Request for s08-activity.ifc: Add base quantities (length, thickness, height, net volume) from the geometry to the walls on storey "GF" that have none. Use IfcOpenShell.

First a look at what the model holds.

```python
import ifcopenshell
import ifcopenshell.util.element
import ifcopenshell.util.unit

model = ifcopenshell.open("s08-activity.ifc")
print(model.schema)
for unit_type in ("LENGTHUNIT", "AREAUNIT", "VOLUMEUNIT"):
    print(unit_type, ifcopenshell.util.unit.calculate_unit_scale(model, unit_type))
storey = next(s for s in model.by_type("IfcBuildingStorey") if s.Name == "GF")
walls = [e for e in ifcopenshell.util.element.get_decomposition(storey) if e.is_a("IfcWall")]
for e in sorted(walls, key=lambda e: e.id()):
    print(e.id(), e.is_a(), e.Name, list(ifcopenshell.util.element.get_psets(e, qtos_only=True)), sep=" | ")
```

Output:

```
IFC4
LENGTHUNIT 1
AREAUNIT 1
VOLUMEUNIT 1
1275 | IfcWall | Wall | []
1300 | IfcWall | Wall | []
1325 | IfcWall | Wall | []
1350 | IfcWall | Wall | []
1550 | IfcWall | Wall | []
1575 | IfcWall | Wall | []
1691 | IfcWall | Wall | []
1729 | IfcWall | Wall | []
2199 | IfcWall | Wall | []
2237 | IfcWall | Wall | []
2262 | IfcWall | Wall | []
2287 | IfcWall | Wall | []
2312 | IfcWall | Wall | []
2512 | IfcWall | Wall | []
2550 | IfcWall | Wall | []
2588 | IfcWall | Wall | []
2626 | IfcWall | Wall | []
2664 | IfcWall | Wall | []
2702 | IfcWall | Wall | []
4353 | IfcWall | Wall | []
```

```python
import ifcopenshell
import ifcopenshell.api.pset
import ifcopenshell.geom
import ifcopenshell.util.element
import ifcopenshell.util.shape
import ifcopenshell.util.unit

model = ifcopenshell.open("s08-activity.ifc")
unit_scale = ifcopenshell.util.unit.calculate_unit_scale(model)
volume_scale = ifcopenshell.util.unit.calculate_unit_scale(model, "VOLUMEUNIT")
settings = ifcopenshell.geom.settings()

storey = next(s for s in model.by_type("IfcBuildingStorey") if s.Name == "GF")
walls = [e for e in ifcopenshell.util.element.get_decomposition(storey) if e.is_a("IfcWall")]

for e in sorted(walls, key=lambda e: e.id()):
    if ifcopenshell.util.element.get_psets(e, qtos_only=True, should_inherit=False):
        continue
    # Geometry comes back in metres, in the element's own axes.
    shape = ifcopenshell.geom.create_shape(settings, e)
    values = {
        "Length": ifcopenshell.util.shape.get_x(shape.geometry) / unit_scale,
        "Width": ifcopenshell.util.shape.get_y(shape.geometry) / unit_scale,
        "Height": ifcopenshell.util.shape.get_z(shape.geometry) / unit_scale,
        "NetVolume": ifcopenshell.util.shape.get_volume(shape.geometry) / volume_scale,
    }
    qto = ifcopenshell.api.pset.add_qto(model, product=e, name="Qto_WallBaseQuantities")
    ifcopenshell.api.pset.edit_qto(model, qto=qto, properties=values)
    print(e.id(), {k: round(v, 3) for k, v in values.items()})

model.write("s08-activity_edited.ifc")
```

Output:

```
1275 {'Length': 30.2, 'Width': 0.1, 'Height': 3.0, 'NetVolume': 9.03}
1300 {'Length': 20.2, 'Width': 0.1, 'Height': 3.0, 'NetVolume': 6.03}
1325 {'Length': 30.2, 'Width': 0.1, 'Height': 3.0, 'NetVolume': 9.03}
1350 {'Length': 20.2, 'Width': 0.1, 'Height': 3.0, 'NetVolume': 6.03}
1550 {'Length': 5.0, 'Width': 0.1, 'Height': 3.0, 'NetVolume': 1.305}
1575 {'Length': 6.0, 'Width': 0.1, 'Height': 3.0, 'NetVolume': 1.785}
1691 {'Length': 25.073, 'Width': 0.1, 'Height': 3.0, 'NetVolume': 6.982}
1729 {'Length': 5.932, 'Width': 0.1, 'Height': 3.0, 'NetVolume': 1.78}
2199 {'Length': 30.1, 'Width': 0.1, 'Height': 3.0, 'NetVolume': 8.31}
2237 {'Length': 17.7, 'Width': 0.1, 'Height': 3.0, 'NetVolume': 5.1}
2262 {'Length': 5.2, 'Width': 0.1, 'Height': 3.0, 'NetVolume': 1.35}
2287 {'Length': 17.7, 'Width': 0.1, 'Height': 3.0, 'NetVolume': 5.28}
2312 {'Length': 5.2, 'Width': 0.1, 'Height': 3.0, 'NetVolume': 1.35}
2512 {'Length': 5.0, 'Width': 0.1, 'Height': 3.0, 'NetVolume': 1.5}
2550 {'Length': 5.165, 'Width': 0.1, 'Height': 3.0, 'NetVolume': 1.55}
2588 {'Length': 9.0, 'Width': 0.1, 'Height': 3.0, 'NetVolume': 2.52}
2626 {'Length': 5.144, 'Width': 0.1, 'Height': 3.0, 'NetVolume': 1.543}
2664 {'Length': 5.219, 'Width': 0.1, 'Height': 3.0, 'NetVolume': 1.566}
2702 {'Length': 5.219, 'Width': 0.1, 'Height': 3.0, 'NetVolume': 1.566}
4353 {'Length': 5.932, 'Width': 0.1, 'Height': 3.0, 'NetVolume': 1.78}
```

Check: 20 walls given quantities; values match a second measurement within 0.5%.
